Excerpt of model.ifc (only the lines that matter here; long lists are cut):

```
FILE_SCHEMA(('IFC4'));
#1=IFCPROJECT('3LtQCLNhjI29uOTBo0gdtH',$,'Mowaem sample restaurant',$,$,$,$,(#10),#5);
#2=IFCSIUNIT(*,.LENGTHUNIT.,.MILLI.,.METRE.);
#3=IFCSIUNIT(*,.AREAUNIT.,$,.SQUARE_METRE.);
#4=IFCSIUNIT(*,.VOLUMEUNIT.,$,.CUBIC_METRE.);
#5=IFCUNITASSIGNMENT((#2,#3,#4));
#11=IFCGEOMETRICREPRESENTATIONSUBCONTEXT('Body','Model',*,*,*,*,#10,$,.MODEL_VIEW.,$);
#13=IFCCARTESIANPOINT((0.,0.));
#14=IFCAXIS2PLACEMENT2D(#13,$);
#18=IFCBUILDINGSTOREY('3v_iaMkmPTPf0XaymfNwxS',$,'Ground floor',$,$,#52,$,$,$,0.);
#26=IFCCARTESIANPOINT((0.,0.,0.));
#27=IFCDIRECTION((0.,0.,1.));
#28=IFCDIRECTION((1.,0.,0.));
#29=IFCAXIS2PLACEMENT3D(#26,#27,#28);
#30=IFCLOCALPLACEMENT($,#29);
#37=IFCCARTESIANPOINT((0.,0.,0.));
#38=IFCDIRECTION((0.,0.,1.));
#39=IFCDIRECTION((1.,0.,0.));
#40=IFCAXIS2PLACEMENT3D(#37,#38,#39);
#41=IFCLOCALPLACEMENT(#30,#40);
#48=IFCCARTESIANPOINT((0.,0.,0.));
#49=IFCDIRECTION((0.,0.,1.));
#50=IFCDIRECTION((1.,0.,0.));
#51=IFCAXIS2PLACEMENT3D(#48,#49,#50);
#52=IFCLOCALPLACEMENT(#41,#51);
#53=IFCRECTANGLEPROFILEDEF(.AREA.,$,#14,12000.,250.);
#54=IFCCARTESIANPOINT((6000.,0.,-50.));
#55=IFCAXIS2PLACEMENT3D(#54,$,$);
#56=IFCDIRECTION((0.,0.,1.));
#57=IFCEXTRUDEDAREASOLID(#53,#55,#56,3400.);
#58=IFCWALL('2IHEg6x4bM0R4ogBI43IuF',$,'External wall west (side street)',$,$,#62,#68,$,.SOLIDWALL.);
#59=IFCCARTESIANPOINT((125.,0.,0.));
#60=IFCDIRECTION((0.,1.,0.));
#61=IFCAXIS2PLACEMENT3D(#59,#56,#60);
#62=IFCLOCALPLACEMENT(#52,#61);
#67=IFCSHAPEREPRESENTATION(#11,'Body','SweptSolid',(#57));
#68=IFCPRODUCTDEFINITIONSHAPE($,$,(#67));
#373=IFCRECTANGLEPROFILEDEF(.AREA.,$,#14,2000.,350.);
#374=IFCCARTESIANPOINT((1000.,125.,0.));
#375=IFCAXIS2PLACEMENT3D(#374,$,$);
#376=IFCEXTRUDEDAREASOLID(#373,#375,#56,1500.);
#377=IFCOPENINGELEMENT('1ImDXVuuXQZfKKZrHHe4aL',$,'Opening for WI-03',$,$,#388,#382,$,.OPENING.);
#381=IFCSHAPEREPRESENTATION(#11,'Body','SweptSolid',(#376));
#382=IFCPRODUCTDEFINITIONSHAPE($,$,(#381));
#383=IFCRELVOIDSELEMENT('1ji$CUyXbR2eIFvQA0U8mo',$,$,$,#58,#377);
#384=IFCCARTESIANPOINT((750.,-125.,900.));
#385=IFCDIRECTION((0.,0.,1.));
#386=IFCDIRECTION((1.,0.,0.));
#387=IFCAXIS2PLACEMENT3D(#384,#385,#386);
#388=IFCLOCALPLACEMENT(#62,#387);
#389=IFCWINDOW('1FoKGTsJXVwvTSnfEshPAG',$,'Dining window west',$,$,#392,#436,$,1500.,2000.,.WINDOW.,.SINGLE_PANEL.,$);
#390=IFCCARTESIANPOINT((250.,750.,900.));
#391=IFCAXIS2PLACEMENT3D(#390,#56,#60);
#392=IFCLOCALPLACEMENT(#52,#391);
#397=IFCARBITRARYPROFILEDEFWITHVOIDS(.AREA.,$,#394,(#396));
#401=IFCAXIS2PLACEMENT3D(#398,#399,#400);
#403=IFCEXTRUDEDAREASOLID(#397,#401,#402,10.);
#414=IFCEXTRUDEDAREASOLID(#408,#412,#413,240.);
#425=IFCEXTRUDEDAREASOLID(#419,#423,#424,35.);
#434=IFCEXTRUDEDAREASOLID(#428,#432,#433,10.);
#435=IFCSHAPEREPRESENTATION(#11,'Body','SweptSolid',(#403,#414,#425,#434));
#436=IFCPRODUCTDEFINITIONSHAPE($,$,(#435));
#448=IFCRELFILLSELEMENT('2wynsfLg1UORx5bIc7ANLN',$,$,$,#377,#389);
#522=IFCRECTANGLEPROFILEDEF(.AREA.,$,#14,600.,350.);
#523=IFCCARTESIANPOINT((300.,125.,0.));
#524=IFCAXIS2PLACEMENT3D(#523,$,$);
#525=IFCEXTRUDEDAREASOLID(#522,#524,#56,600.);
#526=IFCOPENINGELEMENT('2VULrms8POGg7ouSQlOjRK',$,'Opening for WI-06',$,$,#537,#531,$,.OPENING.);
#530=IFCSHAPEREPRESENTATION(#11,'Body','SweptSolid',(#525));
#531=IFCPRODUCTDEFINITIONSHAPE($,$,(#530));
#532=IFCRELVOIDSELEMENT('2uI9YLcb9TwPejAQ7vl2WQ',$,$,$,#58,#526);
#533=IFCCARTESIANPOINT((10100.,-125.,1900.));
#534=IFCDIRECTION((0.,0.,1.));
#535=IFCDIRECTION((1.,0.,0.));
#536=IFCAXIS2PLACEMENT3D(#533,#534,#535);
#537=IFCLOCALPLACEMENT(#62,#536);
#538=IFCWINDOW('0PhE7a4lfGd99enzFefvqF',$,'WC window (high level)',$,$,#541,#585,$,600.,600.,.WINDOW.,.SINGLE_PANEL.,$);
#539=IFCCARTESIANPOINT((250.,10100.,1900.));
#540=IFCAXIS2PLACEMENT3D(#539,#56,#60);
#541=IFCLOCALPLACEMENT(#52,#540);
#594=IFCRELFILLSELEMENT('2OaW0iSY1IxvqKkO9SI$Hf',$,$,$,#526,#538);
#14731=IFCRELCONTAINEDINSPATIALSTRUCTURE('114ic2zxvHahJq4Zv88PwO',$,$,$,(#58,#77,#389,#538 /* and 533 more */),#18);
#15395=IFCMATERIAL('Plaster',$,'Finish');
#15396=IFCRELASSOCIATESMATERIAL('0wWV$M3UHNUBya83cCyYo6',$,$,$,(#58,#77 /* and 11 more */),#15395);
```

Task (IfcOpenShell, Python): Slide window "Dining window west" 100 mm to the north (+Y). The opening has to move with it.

```python
import ifcopenshell
import ifcopenshell.api.geometry
import ifcopenshell.util.placement

model = ifcopenshell.open("model.ifc")

window = model.by_id(389)
opening = window.FillsVoids[0].RelatingOpeningElement
wall = opening.VoidsElements[0].RelatingBuildingElement

wall_matrix = ifcopenshell.util.placement.get_local_placement(wall.ObjectPlacement)
shift = wall_matrix[:3, 0] * 100.0
before = ifcopenshell.util.placement.get_local_placement(window.ObjectPlacement)[:3, 3].copy()

# The window is not placed relative to its opening, so move both.
for product in (opening, window):
    matrix = ifcopenshell.util.placement.get_local_placement(product.ObjectPlacement)
    matrix[:3, 3] += shift
    ifcopenshell.api.geometry.edit_object_placement(model, product=product, matrix=matrix, is_si=False)

after = ifcopenshell.util.placement.get_local_placement(window.ObjectPlacement)[:3, 3]
print("window moved by", (after - before).round(3) + 0.0)

model.write("model-out.ifc")
```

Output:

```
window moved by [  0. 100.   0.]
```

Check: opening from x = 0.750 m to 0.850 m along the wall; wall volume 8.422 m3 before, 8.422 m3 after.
